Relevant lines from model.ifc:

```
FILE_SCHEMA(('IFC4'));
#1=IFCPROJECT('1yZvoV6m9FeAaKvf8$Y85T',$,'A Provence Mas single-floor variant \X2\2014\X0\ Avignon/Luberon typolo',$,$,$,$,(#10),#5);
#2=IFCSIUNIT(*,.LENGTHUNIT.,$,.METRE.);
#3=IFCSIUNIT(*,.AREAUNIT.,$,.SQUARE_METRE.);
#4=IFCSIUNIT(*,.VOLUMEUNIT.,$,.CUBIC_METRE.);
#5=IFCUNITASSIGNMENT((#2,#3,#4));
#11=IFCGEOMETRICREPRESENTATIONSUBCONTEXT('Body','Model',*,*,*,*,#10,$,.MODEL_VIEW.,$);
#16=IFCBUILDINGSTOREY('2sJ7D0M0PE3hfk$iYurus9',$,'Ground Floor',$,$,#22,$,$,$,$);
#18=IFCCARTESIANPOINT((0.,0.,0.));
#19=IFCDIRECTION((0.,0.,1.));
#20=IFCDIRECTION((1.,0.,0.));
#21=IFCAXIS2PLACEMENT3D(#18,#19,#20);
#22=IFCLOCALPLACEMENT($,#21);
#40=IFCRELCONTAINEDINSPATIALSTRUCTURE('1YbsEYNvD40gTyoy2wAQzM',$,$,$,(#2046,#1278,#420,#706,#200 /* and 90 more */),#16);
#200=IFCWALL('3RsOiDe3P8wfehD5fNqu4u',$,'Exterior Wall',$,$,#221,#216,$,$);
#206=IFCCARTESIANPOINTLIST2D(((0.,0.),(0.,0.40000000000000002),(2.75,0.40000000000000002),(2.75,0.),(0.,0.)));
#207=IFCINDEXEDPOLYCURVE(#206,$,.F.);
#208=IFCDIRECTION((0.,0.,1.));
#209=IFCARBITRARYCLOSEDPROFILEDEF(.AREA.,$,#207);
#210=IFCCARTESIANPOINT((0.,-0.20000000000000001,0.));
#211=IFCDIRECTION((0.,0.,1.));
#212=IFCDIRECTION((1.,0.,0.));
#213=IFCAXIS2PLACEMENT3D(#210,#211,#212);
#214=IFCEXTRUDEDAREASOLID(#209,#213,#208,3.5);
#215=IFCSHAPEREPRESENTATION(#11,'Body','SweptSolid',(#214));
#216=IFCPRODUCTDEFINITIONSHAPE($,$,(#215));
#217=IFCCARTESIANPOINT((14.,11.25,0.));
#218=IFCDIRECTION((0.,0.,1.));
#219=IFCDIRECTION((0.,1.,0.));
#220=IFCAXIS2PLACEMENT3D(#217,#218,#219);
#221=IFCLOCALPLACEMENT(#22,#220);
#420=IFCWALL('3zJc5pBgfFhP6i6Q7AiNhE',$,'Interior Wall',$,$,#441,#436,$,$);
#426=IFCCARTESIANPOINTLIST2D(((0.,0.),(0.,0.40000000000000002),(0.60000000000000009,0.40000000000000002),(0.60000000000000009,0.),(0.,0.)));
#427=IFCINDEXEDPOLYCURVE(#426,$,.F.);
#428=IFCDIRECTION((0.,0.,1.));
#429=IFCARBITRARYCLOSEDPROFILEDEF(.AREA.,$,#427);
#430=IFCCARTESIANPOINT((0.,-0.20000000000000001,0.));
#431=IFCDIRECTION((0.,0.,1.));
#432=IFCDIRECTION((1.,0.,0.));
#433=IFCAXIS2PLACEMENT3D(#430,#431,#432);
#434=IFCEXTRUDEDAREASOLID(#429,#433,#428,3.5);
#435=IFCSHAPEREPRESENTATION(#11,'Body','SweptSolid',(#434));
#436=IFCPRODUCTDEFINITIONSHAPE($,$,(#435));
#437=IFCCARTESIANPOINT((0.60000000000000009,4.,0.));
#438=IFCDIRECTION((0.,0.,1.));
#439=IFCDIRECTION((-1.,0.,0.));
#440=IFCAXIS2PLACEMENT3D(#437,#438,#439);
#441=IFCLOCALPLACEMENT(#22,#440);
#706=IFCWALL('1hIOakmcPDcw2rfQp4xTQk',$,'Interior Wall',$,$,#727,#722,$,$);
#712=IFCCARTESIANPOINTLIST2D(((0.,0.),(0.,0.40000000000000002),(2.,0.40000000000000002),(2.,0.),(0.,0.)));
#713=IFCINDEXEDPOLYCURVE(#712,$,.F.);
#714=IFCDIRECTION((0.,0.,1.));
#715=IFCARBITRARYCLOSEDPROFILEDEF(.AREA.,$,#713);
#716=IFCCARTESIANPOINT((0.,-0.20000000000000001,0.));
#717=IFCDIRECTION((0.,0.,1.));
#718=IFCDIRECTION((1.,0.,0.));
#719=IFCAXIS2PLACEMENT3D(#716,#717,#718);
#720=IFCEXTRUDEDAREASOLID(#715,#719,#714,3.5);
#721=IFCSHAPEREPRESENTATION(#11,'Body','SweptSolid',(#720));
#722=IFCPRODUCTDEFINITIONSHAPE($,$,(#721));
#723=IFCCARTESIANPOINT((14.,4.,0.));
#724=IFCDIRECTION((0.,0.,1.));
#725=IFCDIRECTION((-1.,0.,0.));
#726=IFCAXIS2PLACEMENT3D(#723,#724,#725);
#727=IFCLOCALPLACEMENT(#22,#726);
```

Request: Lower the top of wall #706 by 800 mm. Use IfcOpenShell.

```python
import ifcopenshell
import ifcopenshell.geom
import ifcopenshell.util.representation
import ifcopenshell.util.shape

model = ifcopenshell.open("model.ifc")
settings = ifcopenshell.geom.settings()


def volume(element):
    """Net volume in cubic metres, openings subtracted."""
    shape = ifcopenshell.geom.create_shape(settings, element)
    return ifcopenshell.util.shape.get_volume(shape.geometry)


wall = model.by_id(706)
before = volume(wall)

body = ifcopenshell.util.representation.get_representation(wall, "Model", "Body")
solid = body.Items[0]
old_height = solid.Depth
solid.Depth -= 0.8
after = volume(wall)

print(f"height {old_height:g} -> {solid.Depth:g}, volume {before:.3f} -> {after:.3f} m3")

model.write("model_edited.ifc")
```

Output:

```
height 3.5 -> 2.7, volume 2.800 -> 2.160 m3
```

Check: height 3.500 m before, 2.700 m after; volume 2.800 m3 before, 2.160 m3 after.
